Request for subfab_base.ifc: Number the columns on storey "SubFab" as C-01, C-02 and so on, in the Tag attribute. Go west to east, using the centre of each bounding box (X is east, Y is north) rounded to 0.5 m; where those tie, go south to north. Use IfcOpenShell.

First a look at what the model holds.

```python
import ifcopenshell
import ifcopenshell.util.element
import ifcopenshell.util.placement

model = ifcopenshell.open("subfab_base.ifc")
print(model.schema)
storey = next(s for s in model.by_type("IfcBuildingStorey") if s.Name == "SubFab")
columns = [e for e in ifcopenshell.util.element.get_decomposition(storey) if e.is_a("IfcColumn")]
for e in sorted(columns, key=lambda e: e.id()):
    origin = ifcopenshell.util.placement.get_local_placement(e.ObjectPlacement)[:3, 3]
    print(e.id(), e.Tag, e.Name, origin.round(2) + 0.0, sep=" | ")
```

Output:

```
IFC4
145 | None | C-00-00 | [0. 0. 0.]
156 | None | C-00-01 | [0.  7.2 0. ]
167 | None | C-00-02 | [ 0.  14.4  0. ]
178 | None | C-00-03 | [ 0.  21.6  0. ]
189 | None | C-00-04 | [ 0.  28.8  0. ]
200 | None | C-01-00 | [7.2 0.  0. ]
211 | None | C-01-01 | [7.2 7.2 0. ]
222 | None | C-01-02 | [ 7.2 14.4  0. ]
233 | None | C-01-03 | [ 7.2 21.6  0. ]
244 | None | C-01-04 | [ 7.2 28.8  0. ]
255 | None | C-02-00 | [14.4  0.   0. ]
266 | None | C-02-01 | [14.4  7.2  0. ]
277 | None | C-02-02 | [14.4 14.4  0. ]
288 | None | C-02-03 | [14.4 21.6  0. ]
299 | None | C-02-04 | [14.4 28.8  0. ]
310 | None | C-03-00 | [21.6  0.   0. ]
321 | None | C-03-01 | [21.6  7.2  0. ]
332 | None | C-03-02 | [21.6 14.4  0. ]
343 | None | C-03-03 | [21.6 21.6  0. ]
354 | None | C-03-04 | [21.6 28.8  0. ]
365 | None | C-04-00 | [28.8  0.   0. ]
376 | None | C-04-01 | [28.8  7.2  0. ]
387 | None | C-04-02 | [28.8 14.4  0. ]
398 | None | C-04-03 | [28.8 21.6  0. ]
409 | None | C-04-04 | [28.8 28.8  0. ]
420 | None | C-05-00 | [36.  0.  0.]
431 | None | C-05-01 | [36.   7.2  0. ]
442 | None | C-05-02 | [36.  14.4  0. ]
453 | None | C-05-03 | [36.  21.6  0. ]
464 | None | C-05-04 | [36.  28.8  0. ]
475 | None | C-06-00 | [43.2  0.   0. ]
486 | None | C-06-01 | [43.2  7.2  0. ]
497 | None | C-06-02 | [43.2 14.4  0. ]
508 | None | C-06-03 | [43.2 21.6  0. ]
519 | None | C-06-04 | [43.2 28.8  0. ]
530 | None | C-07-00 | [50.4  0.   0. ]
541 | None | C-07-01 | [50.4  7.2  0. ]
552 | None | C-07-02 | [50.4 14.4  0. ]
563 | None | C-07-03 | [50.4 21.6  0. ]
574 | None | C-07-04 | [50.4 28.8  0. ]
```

```python
import ifcopenshell
import ifcopenshell.geom
import ifcopenshell.util.element
import ifcopenshell.util.shape

model = ifcopenshell.open("subfab_base.ifc")
settings = ifcopenshell.geom.settings()
settings.set("use-world-coords", True)


def centre(element):
    shape = ifcopenshell.geom.create_shape(settings, element)
    return ifcopenshell.util.shape.get_bbox_centroid(shape.geometry)


storey = next(s for s in model.by_type("IfcBuildingStorey") if s.Name == "SubFab")
columns = [e for e in ifcopenshell.util.element.get_decomposition(storey) if e.is_a("IfcColumn")]

# Insertion points can sit at a corner or the storey origin, so sort by the geometry (in metres).
centres = {e: centre(e) for e in columns}
columns.sort(key=lambda e: (round(centres[e][0] / 0.5), centres[e][1]))

for i, e in enumerate(columns, start=1):
    number = f"C-{i:02d}"
    e.Tag = number
    print(e.id(), number)

model.write("subfab_base_updated.ifc")
```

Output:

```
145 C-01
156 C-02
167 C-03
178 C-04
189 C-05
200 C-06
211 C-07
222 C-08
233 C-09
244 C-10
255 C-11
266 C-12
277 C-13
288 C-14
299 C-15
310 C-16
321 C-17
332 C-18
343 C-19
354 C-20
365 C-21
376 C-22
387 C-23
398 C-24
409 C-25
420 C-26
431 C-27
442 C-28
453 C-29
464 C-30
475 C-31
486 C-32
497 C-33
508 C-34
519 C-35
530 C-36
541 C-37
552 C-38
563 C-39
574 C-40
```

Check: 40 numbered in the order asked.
